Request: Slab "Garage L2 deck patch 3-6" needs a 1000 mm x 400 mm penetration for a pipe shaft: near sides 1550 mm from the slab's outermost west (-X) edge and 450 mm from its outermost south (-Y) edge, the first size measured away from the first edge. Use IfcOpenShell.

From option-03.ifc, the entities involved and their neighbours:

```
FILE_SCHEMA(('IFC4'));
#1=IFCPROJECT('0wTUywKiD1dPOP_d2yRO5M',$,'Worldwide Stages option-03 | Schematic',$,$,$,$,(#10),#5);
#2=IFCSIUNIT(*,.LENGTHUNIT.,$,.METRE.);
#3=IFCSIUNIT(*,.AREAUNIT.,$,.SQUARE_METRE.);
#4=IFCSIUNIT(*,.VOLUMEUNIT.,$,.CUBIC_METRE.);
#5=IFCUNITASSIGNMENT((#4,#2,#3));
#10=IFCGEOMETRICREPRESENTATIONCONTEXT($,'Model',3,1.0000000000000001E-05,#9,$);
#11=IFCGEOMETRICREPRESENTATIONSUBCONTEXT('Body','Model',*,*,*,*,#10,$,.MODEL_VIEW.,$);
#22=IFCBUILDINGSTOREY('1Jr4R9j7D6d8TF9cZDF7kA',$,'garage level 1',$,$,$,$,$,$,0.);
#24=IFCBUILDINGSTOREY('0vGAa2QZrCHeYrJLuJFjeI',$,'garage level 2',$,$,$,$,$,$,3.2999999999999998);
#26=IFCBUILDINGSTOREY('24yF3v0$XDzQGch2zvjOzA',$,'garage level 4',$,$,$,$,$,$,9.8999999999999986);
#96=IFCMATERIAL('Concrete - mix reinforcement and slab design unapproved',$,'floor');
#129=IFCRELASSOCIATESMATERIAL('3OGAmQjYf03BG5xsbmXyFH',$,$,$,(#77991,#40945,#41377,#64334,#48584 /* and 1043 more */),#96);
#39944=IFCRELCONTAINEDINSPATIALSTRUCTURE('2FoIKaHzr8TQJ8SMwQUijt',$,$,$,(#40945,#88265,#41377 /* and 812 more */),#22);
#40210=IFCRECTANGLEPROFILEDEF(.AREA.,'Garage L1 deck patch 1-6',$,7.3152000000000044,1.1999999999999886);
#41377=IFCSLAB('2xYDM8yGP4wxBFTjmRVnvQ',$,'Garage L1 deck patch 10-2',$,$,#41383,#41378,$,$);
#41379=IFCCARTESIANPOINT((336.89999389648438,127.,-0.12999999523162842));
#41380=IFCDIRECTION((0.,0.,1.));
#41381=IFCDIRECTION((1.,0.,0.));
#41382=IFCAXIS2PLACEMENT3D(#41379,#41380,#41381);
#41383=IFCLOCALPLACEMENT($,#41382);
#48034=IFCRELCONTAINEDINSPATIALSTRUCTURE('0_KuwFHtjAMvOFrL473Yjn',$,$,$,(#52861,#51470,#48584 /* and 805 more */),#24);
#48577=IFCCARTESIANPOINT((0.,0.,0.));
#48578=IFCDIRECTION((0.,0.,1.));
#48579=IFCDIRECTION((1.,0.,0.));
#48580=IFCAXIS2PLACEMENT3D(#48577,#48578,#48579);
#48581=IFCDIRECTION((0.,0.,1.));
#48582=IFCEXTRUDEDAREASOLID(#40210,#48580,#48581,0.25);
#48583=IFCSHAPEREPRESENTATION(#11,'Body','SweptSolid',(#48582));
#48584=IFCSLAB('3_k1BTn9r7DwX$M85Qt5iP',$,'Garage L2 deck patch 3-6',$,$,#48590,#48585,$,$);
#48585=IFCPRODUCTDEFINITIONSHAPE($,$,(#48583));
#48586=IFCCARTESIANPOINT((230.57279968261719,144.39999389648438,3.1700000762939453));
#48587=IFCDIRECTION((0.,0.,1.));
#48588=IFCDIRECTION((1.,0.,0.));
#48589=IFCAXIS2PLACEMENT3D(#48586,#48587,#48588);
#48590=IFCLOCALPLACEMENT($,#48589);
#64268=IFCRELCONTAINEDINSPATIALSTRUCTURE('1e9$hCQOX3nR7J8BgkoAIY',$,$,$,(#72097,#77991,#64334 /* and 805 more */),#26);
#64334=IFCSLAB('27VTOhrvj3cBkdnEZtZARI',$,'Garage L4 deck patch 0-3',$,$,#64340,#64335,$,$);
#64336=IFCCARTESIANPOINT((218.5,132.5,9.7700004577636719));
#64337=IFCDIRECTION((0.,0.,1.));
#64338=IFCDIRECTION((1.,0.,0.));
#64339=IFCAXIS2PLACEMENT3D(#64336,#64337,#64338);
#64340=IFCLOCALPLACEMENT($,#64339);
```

```python
import numpy as np
import ifcopenshell
import ifcopenshell.api.feature
import ifcopenshell.api.geometry
import ifcopenshell.api.root
import ifcopenshell.geom
import ifcopenshell.util.placement
import ifcopenshell.util.representation
import ifcopenshell.util.shape
import ifcopenshell.util.unit

model = ifcopenshell.open("option-03.ifc")
unit_scale = ifcopenshell.util.unit.calculate_unit_scale(model)
settings = ifcopenshell.geom.settings()


def volume(element):
    """Net volume in cubic metres, openings subtracted."""
    shape = ifcopenshell.geom.create_shape(settings, element)
    return ifcopenshell.util.shape.get_volume(shape.geometry)


slab = model.by_guid("3_k1BTn9r7DwX$M85Qt5iP")
before = volume(slab)

# Extent in the slab's own axes, in metres. The edges named are its -X and -Y sides.
slab_shape = ifcopenshell.geom.create_shape(settings, slab)
vertices = ifcopenshell.util.shape.get_vertices(slab_shape.geometry)
x_min, y_min, bottom = vertices.min(axis=0)
top = vertices[:, 2].max()

opening = ifcopenshell.api.root.create_entity(model, ifc_class="IfcOpeningElement", name="Pipe shaft opening", predefined_type="OPENING")
context = ifcopenshell.util.representation.get_context(model, "Model", "Body", "MODEL_VIEW")
width, depth = 1, 0.4
outline = [(0.0, 0.0), (width, 0.0), (width, depth), (0.0, depth), (0.0, 0.0)]
# Overshoot both faces by 50 mm so the cut is clean.
shape = ifcopenshell.api.geometry.add_slab_representation(
    model, context=context, depth=top - bottom + 0.1, polyline=outline
)
ifcopenshell.api.geometry.assign_representation(model, product=opening, representation=shape)

matrix = ifcopenshell.util.placement.get_local_placement(slab.ObjectPlacement)
matrix[:, 3] = matrix @ np.append(np.array([x_min + 1.55, y_min + 0.45, bottom - 0.05]) / unit_scale, 1.0)
ifcopenshell.api.geometry.edit_object_placement(model, product=opening, matrix=matrix, is_si=False)
ifcopenshell.api.feature.add_feature(model, feature=opening, element=slab)

after = volume(slab)

print(f"slab volume {before:.3f} -> {after:.3f} m3")

model.write("option-03_v2.ifc")
```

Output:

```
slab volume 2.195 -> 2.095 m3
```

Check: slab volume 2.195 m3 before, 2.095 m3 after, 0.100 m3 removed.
